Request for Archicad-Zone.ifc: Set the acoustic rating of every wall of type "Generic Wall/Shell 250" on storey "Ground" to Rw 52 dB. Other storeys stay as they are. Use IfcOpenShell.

First a look at what the model holds.

```python
import ifcopenshell
import ifcopenshell.util.element

model = ifcopenshell.open("Archicad-Zone.ifc")
print(model.schema)
storey = next(s for s in model.by_type("IfcBuildingStorey") if s.Name == "Ground")
walls = [e for e in ifcopenshell.util.element.get_decomposition(storey) if e.is_a("IfcWall")]
seen = {}
for e in walls:
    element_type = ifcopenshell.util.element.get_type(e)
    key = (element_type.Name if element_type != e and element_type else None, ifcopenshell.util.element.get_pset(e, "Pset_WallCommon", "AcousticRating"))
    seen[key] = seen.get(key, 0) + 1
for (name, value), count in sorted(seen.items(), key=str):
    print(count, "x", name, "|", value)
```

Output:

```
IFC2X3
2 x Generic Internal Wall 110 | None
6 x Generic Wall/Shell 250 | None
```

```python
import ifcopenshell
import ifcopenshell.api.pset
import ifcopenshell.util.element

model = ifcopenshell.open("Archicad-Zone.ifc")

storey = next(s for s in model.by_type("IfcBuildingStorey") if s.Name == "Ground")
walls = [e for e in ifcopenshell.util.element.get_decomposition(storey) if e.is_a("IfcWall")]

count = 0
for e in walls:
    element_type = ifcopenshell.util.element.get_type(e)
    if element_type in (None, e) or element_type.Name != "Generic Wall/Shell 250":
        continue
    # add_pset returns the element's existing set when there is one.
    pset = ifcopenshell.api.pset.add_pset(model, product=e, name="Pset_WallCommon")
    ifcopenshell.api.pset.edit_pset(model, pset=pset, properties={"AcousticRating": "Rw 52 dB"})
    count += 1

print(count, "walls updated")

model.write("Archicad-Zone_updated.ifc")
```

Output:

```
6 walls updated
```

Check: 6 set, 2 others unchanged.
